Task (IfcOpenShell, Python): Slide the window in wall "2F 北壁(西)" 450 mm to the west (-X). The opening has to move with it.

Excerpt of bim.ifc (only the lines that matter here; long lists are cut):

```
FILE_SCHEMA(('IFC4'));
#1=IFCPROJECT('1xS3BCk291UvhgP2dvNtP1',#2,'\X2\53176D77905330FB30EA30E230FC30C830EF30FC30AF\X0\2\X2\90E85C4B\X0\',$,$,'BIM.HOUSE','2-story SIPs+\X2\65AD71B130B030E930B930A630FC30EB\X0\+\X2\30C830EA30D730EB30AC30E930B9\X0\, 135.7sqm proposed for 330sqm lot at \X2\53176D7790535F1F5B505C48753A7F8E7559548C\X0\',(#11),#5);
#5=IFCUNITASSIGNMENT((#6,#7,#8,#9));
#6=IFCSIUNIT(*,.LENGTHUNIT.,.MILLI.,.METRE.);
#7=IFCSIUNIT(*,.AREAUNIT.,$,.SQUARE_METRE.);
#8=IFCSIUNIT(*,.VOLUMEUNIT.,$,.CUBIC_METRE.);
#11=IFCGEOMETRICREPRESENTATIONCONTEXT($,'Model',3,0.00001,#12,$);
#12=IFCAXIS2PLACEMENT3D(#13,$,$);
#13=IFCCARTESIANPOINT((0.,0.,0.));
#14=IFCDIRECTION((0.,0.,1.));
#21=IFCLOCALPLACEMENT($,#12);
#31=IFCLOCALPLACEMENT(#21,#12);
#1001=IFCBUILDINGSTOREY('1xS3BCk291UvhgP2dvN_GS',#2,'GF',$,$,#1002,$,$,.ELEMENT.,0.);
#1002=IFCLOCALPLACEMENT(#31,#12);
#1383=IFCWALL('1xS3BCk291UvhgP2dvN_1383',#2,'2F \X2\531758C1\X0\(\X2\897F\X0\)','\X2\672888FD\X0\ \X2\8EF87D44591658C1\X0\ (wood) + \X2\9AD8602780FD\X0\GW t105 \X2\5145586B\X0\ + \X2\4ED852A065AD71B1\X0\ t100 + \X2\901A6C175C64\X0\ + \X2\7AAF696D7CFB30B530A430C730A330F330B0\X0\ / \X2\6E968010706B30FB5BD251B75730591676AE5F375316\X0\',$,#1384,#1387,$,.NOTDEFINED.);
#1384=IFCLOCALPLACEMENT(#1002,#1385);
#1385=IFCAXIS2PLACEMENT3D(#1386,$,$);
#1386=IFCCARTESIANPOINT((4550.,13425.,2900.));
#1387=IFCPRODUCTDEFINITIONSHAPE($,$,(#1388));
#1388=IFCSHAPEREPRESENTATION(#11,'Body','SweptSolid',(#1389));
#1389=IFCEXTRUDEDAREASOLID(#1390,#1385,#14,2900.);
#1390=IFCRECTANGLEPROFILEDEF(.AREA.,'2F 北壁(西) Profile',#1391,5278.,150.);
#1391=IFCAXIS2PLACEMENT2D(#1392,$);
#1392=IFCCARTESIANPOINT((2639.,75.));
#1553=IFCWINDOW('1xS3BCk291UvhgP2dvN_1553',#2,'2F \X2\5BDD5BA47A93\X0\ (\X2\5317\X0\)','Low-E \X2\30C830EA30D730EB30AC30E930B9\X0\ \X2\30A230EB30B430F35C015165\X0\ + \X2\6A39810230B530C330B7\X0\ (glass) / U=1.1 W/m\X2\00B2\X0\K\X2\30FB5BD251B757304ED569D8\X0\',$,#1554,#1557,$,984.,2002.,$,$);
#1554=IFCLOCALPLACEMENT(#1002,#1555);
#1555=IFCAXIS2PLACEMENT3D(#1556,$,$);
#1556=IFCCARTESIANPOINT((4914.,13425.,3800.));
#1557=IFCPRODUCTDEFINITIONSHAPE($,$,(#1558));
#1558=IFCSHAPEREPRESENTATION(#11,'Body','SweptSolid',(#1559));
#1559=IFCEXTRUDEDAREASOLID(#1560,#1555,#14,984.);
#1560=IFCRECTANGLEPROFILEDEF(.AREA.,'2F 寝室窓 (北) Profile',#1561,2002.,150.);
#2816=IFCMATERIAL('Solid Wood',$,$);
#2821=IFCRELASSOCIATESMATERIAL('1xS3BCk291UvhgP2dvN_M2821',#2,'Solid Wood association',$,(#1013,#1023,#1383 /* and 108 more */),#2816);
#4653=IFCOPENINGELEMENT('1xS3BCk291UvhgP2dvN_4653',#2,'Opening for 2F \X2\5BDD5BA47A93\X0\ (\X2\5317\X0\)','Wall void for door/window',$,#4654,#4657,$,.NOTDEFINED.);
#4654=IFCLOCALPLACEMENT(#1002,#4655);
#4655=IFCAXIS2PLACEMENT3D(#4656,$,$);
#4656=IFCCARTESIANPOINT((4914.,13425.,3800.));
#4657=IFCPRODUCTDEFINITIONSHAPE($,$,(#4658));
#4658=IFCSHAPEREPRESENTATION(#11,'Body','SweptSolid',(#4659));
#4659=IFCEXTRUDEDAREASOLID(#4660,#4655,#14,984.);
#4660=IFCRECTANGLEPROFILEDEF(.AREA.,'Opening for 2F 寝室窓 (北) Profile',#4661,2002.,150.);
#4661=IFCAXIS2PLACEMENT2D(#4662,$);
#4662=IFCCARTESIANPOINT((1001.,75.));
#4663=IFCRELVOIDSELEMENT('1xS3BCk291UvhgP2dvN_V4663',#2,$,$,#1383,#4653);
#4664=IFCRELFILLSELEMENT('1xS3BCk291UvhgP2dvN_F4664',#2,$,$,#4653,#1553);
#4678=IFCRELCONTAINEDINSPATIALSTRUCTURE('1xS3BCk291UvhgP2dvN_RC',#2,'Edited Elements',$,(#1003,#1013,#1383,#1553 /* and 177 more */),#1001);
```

```python
import ifcopenshell
import ifcopenshell.api.geometry
import ifcopenshell.util.placement
import ifcopenshell.util.unit

model = ifcopenshell.open("bim.ifc")
unit_scale = ifcopenshell.util.unit.calculate_unit_scale(model)

window = model.by_guid("1xS3BCk291UvhgP2dvN_1553")
opening = window.FillsVoids[0].RelatingOpeningElement
wall = opening.VoidsElements[0].RelatingBuildingElement

wall_matrix = ifcopenshell.util.placement.get_local_placement(wall.ObjectPlacement)
shift = wall_matrix[:3, 0] * -0.45 / unit_scale
before = ifcopenshell.util.placement.get_local_placement(window.ObjectPlacement)[:3, 3].copy()

# The window is not placed relative to its opening, so move both.
for product in (opening, window):
    matrix = ifcopenshell.util.placement.get_local_placement(product.ObjectPlacement)
    matrix[:3, 3] += shift
    ifcopenshell.api.geometry.edit_object_placement(model, product=product, matrix=matrix, is_si=False)

after = ifcopenshell.util.placement.get_local_placement(window.ObjectPlacement)[:3, 3]
print("window moved by", (after - before).round(3) + 0.0)

model.write("bim_updated.ifc")
```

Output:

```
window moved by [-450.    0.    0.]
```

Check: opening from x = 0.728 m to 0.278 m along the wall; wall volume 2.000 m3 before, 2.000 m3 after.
